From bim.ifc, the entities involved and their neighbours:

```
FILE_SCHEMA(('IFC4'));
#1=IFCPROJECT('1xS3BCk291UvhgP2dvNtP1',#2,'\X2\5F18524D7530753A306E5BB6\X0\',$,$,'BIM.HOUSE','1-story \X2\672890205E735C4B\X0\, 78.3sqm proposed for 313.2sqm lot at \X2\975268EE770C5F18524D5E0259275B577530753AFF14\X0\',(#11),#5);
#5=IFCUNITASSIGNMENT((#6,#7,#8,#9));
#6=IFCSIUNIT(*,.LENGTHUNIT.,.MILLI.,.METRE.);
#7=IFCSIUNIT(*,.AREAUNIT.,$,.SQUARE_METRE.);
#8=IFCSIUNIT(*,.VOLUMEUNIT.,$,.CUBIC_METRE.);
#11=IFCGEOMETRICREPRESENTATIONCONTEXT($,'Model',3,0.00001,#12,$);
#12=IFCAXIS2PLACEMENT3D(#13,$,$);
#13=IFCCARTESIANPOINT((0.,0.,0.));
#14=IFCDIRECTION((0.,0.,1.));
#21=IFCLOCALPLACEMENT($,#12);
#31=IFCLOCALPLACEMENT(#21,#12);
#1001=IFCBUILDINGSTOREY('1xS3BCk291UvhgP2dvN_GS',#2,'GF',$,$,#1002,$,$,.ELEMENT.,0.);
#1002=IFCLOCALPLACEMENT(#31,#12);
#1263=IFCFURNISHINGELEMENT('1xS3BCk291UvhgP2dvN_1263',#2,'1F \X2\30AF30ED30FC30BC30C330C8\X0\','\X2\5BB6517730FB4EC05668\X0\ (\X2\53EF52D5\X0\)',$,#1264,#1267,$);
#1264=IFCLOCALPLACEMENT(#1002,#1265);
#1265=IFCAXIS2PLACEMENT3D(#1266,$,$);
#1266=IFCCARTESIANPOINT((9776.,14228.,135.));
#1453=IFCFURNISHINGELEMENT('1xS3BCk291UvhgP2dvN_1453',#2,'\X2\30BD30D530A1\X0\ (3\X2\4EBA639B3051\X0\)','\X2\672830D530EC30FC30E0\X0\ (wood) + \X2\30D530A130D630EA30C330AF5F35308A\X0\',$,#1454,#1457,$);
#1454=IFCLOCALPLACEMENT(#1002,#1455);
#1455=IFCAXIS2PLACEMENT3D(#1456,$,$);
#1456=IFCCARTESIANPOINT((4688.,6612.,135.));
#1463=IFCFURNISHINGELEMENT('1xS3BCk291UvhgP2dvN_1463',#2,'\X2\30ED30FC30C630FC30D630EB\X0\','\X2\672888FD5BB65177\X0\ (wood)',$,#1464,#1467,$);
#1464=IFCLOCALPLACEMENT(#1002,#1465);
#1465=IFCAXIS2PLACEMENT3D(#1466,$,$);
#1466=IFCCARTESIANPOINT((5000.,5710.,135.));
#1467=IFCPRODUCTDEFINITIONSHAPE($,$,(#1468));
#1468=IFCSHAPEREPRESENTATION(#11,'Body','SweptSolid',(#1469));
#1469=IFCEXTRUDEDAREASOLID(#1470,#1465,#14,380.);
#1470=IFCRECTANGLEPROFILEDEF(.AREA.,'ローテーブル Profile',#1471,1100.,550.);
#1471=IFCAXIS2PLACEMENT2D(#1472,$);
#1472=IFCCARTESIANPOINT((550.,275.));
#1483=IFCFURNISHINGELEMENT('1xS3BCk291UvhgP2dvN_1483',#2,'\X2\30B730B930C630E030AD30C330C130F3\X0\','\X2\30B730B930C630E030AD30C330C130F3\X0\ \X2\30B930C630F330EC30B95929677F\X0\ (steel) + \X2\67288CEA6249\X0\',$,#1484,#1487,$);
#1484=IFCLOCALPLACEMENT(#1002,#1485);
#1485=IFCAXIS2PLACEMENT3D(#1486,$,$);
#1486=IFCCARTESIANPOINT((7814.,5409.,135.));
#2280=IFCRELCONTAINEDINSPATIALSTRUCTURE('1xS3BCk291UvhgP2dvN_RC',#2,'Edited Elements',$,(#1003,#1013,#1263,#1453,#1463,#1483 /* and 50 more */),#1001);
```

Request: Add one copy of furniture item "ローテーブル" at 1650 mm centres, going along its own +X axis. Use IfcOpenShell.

```python
import ifcopenshell
import ifcopenshell.api.geometry
import ifcopenshell.api.root
import ifcopenshell.util.element
import ifcopenshell.util.placement
import ifcopenshell.util.unit

model = ifcopenshell.open("bim.ifc")
unit_scale = ifcopenshell.util.unit.calculate_unit_scale(model)


def reuse_history(source, copy):
    """copy_class also copies each property set's owner history, people and application; keep the originals."""
    for rel in copy.IsDefinedBy:
        if rel.is_a("IfcRelDefinesByProperties") and (history := rel.RelatingPropertyDefinition.OwnerHistory):
            rel.RelatingPropertyDefinition.OwnerHistory = source.OwnerHistory
            ifcopenshell.util.element.remove_deep2(model, history)


source = model.by_guid("1xS3BCk291UvhgP2dvN_1463")
base = ifcopenshell.util.placement.get_local_placement(source.ObjectPlacement)
step = base[:3, 0] * 1.65 / unit_scale

for i in range(1, 2):
    copy = ifcopenshell.api.root.copy_class(model, product=source)
    copy.Representation = ifcopenshell.util.element.copy_deep(
        model, source.Representation, exclude=["IfcGeometricRepresentationContext", "IfcRepresentationMap"]
    )
    reuse_history(source, copy)
    matrix = base.copy()
    matrix[:3, 3] += i * step
    print("added at", matrix[:3, 3].round(3) + 0.0)
    ifcopenshell.api.geometry.edit_object_placement(model, product=copy, matrix=matrix, is_si=False)

model.write("bim_v2.ifc")
```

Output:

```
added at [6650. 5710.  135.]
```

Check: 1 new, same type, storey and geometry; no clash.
